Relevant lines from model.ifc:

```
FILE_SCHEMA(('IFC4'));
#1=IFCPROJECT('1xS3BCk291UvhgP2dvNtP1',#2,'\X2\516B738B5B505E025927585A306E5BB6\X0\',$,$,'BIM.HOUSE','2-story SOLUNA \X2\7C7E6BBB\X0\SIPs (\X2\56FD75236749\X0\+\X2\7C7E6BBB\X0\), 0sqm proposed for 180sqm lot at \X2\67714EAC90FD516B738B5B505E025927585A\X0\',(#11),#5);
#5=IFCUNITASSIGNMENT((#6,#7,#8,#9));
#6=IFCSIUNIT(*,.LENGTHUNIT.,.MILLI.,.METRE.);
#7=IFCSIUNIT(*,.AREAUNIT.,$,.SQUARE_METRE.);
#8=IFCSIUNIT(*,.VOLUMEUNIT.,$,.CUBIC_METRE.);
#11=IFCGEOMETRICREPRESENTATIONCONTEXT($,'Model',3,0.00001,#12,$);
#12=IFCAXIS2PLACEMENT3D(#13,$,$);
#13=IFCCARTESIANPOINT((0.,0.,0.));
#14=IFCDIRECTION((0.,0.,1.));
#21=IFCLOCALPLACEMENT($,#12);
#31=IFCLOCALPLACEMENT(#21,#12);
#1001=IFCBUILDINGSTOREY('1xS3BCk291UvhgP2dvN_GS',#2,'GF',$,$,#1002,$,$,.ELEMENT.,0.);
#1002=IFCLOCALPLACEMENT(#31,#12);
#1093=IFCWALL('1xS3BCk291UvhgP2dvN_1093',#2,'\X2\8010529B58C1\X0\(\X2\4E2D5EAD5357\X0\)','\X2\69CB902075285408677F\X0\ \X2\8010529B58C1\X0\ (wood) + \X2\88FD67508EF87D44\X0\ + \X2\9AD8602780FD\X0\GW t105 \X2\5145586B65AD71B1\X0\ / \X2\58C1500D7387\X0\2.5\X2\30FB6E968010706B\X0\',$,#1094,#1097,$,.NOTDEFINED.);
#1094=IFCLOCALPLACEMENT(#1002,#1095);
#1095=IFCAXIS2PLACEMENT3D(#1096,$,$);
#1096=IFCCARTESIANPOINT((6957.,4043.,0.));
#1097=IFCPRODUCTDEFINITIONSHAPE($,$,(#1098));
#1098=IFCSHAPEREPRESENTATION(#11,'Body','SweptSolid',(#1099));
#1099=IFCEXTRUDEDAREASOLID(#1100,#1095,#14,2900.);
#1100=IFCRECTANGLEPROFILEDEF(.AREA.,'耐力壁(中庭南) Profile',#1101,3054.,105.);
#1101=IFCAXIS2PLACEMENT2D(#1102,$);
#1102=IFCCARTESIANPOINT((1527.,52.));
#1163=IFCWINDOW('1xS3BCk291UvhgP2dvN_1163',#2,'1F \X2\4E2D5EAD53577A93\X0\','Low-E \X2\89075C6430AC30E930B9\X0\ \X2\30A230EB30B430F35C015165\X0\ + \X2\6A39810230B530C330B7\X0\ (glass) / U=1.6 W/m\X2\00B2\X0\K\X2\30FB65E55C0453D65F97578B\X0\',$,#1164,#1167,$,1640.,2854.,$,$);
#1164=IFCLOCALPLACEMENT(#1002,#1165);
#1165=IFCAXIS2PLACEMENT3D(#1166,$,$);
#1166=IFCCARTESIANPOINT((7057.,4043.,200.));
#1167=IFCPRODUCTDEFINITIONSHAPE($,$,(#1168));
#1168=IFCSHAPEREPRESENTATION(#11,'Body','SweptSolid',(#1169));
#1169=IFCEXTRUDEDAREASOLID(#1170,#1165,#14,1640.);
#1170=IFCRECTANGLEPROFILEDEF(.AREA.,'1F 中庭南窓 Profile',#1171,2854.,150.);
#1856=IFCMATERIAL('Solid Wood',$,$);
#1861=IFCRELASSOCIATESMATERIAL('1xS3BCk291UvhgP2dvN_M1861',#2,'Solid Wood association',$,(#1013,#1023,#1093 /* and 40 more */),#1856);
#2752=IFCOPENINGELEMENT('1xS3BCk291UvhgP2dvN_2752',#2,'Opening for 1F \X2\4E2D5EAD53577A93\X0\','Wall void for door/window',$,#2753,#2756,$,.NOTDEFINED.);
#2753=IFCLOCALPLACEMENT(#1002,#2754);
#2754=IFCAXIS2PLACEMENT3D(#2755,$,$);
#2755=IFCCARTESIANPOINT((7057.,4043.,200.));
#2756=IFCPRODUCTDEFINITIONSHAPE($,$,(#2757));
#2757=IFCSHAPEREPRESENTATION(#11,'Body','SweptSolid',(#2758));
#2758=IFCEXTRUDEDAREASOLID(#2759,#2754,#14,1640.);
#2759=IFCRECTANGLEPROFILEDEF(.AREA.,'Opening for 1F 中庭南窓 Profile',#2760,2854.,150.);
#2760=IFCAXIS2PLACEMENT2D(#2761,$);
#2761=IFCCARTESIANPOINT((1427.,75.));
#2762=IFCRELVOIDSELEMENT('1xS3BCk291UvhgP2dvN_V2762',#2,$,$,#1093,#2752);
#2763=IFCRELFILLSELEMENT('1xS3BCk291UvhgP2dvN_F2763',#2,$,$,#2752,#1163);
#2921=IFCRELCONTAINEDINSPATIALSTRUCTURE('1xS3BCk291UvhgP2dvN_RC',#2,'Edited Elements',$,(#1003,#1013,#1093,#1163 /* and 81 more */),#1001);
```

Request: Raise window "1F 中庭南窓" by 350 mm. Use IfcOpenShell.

```python
import numpy as np
import ifcopenshell
import ifcopenshell.api.geometry
import ifcopenshell.util.placement
import ifcopenshell.util.unit

model = ifcopenshell.open("model.ifc")
unit_scale = ifcopenshell.util.unit.calculate_unit_scale(model)

window = model.by_guid("1xS3BCk291UvhgP2dvN_1163")
opening = window.FillsVoids[0].RelatingOpeningElement
dz = 350.0

shift = np.array([0.0, 0.0, dz])
# The window is not placed relative to its opening, so move both.
for product in (opening, window):
    matrix = ifcopenshell.util.placement.get_local_placement(product.ObjectPlacement)
    matrix[:3, 3] += shift
    ifcopenshell.api.geometry.edit_object_placement(model, product=product, matrix=matrix, is_si=False)

print(f"moved by {dz * unit_scale:+.3f} m")

model.write("model_edited.ifc")
```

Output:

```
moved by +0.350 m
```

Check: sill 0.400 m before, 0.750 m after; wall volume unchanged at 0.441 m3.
